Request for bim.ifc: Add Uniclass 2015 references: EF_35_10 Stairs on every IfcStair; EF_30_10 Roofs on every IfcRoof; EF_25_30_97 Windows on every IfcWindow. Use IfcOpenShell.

First a look at what the model holds.

```python
import ifcopenshell

model = ifcopenshell.open("bim.ifc")
print(model.schema)
print("classifications:", [c.Name for c in model.by_type("IfcClassification")])
for ifc_class in ("IfcDoor", "IfcRoof", "IfcStair", "IfcWall", "IfcWindow"):
    print(ifc_class, len(model.by_type(ifc_class)))
```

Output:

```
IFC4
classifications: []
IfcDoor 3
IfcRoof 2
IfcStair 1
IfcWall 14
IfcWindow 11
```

```python
import ifcopenshell
import ifcopenshell.api.classification

model = ifcopenshell.open("bim.ifc")

system = ifcopenshell.api.classification.add_classification(model, classification="Uniclass 2015")

codes = {
    "IfcStair": ("EF_35_10", "Stairs"),
    "IfcRoof": ("EF_30_10", "Roofs"),
    "IfcWindow": ("EF_25_30_97", "Windows"),
}
for ifc_class, (code, name) in codes.items():
    products = model.by_type(ifc_class)
    ifcopenshell.api.classification.add_reference(
        model, products=products, classification=system, identification=code, name=name
    )
    print(code, len(products))

model.write("bim-out.ifc")
```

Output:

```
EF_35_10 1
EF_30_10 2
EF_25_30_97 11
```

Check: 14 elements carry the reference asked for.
